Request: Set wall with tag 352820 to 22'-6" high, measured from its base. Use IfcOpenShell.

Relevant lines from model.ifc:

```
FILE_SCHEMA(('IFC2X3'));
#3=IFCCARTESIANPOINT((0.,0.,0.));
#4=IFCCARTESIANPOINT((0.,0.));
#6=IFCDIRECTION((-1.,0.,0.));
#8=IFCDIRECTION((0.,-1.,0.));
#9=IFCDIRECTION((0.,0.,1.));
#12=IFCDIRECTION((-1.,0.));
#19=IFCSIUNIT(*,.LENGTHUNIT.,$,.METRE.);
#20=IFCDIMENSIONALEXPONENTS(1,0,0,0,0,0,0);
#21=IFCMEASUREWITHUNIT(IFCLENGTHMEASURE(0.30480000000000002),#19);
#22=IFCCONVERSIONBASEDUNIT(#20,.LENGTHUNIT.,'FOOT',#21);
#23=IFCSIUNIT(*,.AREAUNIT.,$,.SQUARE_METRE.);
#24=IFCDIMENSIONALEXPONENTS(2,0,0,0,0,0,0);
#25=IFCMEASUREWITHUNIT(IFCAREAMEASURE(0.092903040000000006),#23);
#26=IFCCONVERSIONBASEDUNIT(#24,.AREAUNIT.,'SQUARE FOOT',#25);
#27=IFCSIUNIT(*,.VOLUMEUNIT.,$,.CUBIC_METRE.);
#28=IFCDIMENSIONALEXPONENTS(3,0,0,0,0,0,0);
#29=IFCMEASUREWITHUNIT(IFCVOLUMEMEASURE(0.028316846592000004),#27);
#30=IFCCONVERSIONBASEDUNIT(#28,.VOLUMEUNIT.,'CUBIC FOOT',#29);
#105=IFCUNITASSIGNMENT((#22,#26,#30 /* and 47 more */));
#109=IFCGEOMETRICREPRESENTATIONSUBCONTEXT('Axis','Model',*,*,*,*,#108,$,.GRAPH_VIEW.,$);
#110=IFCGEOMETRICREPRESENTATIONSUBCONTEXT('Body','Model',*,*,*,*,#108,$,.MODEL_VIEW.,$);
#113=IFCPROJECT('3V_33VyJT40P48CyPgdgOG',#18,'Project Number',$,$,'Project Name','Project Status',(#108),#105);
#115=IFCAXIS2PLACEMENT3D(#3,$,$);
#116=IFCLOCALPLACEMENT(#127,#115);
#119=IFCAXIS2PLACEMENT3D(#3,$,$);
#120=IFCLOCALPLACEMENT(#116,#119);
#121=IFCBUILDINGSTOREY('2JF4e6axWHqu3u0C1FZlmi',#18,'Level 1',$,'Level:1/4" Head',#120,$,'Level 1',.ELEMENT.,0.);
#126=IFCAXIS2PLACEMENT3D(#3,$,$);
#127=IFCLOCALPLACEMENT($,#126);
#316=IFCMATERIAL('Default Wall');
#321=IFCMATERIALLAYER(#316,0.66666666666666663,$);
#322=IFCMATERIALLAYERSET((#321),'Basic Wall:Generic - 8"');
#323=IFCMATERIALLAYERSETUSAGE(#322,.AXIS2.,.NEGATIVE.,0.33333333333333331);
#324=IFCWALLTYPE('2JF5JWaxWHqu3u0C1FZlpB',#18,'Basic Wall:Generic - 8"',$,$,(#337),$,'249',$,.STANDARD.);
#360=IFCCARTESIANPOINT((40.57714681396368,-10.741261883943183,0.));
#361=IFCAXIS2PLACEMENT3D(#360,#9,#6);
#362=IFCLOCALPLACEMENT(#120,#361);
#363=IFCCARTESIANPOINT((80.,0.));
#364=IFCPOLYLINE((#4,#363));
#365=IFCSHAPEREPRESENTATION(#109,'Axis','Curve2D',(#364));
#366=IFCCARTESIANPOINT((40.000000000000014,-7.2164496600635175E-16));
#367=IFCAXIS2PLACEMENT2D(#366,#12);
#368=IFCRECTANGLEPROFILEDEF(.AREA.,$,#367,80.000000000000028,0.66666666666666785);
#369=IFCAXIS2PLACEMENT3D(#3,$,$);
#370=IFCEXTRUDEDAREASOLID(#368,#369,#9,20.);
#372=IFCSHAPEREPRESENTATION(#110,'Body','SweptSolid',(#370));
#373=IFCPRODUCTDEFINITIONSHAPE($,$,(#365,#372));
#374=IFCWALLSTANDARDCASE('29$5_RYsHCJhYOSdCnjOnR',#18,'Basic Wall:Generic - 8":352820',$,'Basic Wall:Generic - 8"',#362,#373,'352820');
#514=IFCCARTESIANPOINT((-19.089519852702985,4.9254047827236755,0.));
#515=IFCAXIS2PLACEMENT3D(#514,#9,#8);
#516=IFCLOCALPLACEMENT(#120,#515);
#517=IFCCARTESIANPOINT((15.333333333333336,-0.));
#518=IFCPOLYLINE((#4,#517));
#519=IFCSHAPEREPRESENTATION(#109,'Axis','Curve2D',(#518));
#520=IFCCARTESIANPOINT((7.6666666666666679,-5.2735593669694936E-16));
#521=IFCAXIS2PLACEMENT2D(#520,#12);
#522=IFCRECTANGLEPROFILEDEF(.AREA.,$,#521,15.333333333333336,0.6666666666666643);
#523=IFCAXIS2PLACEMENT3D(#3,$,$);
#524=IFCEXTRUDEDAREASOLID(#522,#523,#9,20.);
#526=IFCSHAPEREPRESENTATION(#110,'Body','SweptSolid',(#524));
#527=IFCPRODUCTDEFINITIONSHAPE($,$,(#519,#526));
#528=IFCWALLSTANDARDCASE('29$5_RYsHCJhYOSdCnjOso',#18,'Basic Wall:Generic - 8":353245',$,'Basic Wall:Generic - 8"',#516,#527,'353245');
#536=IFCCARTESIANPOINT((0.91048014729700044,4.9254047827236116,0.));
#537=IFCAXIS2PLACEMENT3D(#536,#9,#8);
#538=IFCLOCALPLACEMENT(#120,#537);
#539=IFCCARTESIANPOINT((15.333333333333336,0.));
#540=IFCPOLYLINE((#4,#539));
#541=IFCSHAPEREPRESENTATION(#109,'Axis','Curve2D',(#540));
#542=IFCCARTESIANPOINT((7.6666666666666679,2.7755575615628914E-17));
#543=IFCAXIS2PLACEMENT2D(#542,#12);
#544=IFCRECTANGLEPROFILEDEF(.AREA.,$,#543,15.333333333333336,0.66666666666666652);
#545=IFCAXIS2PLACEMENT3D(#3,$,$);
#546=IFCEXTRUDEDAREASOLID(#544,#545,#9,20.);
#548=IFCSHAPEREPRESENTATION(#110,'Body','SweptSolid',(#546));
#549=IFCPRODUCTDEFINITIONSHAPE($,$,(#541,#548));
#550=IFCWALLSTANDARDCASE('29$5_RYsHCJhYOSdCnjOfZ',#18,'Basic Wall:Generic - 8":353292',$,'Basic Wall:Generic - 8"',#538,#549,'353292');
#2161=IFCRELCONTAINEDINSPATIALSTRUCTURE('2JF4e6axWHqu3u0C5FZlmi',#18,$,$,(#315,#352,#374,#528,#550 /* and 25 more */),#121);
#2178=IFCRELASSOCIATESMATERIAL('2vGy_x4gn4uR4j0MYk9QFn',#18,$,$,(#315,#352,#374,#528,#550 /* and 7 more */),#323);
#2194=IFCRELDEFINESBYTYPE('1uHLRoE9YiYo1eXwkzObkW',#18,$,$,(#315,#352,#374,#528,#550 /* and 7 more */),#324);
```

```python
import ifcopenshell
import ifcopenshell.geom
import ifcopenshell.util.representation
import ifcopenshell.util.shape
import ifcopenshell.util.unit

model = ifcopenshell.open("model.ifc")
unit_scale = ifcopenshell.util.unit.calculate_unit_scale(model)
settings = ifcopenshell.geom.settings()


def volume(element):
    """Net volume in cubic metres, openings subtracted."""
    shape = ifcopenshell.geom.create_shape(settings, element)
    return ifcopenshell.util.shape.get_volume(shape.geometry)


wall = model.by_guid("29$5_RYsHCJhYOSdCnjOnR")
before = volume(wall)

body = ifcopenshell.util.representation.get_representation(wall, "Model", "Body")
solid = body.Items[0]
old_height = solid.Depth
solid.Depth = 270 * 0.0254 / unit_scale
after = volume(wall)

print(f"height {old_height:g} -> {solid.Depth:g}, volume {before:.3f} -> {after:.3f} m3")

model.write("model-out.ifc")
```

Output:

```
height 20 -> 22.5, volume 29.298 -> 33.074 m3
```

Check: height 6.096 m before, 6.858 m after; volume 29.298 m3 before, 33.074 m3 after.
